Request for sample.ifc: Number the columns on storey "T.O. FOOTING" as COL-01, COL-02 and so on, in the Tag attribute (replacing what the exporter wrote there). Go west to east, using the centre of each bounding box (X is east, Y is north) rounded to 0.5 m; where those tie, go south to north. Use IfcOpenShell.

First a look at what the model holds.

```python
import ifcopenshell
import ifcopenshell.util.element
import ifcopenshell.util.placement

model = ifcopenshell.open("sample.ifc")
print(model.schema)
storey = next(s for s in model.by_type("IfcBuildingStorey") if s.Name == "T.O. FOOTING")
columns = [e for e in ifcopenshell.util.element.get_decomposition(storey) if e.is_a("IfcColumn")]
for e in sorted(columns, key=lambda e: e.id()):
    origin = ifcopenshell.util.placement.get_local_placement(e.ObjectPlacement)[:3, 3]
    print(e.id(), e.Tag, e.Name, origin.round(2) + 0.0, sep=" | ")
```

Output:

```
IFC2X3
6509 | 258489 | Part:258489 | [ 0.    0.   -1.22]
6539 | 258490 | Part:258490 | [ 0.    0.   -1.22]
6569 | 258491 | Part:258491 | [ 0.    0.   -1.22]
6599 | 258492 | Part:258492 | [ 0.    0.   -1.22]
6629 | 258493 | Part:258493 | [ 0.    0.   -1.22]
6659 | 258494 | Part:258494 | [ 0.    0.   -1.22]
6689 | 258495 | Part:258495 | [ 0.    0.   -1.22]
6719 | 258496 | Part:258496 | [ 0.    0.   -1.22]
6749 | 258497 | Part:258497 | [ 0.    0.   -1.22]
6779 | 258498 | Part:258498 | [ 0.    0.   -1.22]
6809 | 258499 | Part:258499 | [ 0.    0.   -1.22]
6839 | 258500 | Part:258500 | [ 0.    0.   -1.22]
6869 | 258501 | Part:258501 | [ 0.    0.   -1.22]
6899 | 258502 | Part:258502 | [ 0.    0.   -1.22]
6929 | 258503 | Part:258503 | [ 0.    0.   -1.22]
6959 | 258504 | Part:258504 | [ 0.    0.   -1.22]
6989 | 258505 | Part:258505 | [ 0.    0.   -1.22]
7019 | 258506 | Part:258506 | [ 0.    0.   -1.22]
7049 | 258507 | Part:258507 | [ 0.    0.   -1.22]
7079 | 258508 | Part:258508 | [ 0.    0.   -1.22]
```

```python
import ifcopenshell
import ifcopenshell.geom
import ifcopenshell.util.element
import ifcopenshell.util.shape

model = ifcopenshell.open("sample.ifc")
settings = ifcopenshell.geom.settings()
settings.set("use-world-coords", True)


def centre(element):
    shape = ifcopenshell.geom.create_shape(settings, element)
    return ifcopenshell.util.shape.get_bbox_centroid(shape.geometry)


storey = next(s for s in model.by_type("IfcBuildingStorey") if s.Name == "T.O. FOOTING")
columns = [e for e in ifcopenshell.util.element.get_decomposition(storey) if e.is_a("IfcColumn")]

# Insertion points can sit at a corner or the storey origin, so sort by the geometry (in metres).
centres = {e: centre(e) for e in columns}
columns.sort(key=lambda e: (round(centres[e][0] / 0.5), centres[e][1]))

for i, e in enumerate(columns, start=1):
    number = f"COL-{i:02d}"
    e.Tag = number
    print(e.id(), number)

model.write("sample_v2.ifc")
```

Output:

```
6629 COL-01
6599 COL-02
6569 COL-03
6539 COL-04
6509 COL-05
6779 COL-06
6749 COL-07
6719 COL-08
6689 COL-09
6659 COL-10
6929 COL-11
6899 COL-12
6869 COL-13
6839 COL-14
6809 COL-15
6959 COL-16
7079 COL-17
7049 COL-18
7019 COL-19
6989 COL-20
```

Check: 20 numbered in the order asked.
